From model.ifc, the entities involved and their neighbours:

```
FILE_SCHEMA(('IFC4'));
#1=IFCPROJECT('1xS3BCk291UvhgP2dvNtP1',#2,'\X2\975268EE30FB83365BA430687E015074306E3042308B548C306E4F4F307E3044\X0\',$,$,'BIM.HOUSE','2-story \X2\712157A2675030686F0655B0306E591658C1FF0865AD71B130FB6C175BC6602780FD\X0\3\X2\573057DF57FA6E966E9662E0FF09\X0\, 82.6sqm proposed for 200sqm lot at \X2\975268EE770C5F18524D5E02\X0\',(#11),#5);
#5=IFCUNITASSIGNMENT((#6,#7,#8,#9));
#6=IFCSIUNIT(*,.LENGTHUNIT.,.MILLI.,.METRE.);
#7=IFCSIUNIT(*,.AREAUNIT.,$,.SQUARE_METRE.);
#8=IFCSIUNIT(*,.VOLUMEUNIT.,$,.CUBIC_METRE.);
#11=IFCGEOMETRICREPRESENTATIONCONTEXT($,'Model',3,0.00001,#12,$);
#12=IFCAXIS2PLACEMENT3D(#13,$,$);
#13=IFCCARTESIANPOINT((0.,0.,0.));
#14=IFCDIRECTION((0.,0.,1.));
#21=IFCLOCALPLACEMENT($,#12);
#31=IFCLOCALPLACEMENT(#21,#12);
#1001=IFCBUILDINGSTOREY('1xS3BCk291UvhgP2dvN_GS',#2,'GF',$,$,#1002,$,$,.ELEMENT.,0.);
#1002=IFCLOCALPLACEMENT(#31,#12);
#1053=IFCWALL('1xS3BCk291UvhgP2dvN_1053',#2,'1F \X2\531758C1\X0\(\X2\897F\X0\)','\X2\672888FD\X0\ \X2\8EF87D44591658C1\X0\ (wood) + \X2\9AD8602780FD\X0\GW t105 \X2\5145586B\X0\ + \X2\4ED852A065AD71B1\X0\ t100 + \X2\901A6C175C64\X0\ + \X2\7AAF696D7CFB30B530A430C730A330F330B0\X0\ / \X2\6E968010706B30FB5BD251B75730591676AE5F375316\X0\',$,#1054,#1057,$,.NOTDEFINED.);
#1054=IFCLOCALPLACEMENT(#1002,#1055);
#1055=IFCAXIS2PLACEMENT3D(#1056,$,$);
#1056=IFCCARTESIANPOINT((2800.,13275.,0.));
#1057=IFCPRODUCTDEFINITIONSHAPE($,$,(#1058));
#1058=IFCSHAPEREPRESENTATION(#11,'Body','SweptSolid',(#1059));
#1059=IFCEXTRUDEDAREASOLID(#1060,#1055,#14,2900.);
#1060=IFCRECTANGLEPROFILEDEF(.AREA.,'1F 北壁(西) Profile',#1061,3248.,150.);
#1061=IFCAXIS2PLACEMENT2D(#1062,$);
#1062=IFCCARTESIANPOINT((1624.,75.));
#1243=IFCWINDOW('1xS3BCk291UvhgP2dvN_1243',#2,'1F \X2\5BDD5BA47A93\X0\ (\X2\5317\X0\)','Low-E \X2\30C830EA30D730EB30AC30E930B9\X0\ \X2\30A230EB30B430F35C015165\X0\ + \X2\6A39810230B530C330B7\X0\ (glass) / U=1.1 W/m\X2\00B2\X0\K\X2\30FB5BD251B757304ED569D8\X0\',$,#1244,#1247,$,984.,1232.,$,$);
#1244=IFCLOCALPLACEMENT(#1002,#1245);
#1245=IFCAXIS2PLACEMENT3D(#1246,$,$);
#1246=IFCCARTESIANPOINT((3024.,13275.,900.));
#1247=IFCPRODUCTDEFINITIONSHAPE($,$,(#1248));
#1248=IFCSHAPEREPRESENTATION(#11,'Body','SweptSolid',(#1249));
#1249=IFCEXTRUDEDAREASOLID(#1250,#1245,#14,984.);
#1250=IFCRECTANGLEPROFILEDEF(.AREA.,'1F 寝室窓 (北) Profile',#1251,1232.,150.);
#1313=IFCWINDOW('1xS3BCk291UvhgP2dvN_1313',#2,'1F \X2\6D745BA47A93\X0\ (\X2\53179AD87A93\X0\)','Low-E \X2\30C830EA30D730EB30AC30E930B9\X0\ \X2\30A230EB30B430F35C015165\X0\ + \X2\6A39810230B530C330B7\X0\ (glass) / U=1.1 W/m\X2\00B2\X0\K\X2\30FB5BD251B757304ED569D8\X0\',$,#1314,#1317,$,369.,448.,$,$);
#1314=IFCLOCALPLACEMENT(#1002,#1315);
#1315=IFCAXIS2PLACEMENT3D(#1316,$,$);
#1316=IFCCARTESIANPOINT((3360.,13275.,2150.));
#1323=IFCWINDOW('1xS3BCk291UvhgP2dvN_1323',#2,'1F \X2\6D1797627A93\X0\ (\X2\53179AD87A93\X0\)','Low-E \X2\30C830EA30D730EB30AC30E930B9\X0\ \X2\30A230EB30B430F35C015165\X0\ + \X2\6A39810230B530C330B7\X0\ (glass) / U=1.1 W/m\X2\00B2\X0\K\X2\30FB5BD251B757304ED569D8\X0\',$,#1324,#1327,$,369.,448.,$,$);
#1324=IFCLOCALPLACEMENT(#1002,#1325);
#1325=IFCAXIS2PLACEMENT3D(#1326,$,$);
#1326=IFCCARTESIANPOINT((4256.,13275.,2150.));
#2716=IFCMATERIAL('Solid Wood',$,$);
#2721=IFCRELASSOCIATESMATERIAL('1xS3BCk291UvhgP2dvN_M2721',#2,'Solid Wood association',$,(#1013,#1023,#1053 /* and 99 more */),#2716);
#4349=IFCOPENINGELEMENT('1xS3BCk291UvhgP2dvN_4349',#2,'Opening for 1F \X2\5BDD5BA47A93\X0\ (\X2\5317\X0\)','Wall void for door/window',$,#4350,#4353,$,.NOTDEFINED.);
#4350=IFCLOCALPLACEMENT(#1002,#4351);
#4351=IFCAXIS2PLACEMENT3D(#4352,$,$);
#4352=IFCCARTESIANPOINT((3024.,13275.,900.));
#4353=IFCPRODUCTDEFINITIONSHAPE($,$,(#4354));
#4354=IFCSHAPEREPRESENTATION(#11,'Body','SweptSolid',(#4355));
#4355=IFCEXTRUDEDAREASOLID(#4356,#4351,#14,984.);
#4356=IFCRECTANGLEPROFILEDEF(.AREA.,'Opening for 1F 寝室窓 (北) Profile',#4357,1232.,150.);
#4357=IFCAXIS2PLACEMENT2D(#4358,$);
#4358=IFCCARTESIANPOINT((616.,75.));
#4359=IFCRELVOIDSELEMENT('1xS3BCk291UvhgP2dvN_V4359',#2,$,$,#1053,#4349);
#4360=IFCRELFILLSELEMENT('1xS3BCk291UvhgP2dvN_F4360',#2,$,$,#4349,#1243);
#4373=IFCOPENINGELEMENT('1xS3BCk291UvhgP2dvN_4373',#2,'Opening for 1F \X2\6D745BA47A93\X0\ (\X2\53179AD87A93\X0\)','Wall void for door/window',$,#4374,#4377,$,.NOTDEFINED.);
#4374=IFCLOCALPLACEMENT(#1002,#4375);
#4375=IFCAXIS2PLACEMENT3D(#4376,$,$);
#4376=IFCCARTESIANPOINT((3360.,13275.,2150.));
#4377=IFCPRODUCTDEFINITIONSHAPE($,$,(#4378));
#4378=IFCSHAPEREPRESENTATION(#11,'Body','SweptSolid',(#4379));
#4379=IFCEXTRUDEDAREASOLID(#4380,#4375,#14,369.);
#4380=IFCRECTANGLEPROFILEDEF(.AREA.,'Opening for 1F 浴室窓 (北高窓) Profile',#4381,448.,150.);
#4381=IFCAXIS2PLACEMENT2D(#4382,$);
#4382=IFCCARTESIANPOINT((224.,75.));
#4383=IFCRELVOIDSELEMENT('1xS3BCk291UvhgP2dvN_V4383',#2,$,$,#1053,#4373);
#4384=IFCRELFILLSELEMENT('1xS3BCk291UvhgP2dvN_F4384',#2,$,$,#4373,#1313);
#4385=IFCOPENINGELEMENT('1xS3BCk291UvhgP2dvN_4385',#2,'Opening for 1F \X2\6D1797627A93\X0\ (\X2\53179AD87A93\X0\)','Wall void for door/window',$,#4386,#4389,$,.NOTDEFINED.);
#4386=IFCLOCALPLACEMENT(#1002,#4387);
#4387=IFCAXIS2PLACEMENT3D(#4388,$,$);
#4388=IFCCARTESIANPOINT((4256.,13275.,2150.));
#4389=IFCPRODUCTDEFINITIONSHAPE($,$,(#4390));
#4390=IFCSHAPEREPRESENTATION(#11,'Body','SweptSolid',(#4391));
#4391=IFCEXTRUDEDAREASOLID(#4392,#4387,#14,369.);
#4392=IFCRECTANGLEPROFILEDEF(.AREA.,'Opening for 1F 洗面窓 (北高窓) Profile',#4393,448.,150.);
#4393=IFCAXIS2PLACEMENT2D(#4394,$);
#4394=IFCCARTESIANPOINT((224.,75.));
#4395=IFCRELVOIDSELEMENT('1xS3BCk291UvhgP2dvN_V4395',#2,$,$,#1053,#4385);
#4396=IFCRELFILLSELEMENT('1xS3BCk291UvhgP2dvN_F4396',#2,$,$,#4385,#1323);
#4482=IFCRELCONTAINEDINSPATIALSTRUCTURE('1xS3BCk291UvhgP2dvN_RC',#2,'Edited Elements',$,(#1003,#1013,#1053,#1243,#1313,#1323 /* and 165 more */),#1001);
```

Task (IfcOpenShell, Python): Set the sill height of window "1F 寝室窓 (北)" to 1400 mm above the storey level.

```python
import numpy as np
import ifcopenshell
import ifcopenshell.api.geometry
import ifcopenshell.geom
import ifcopenshell.util.element
import ifcopenshell.util.placement
import ifcopenshell.util.shape
import ifcopenshell.util.unit

model = ifcopenshell.open("model.ifc")
unit_scale = ifcopenshell.util.unit.calculate_unit_scale(model)

window = model.by_id(1243)
opening = window.FillsVoids[0].RelatingOpeningElement
storey = ifcopenshell.util.element.get_container(window, ifc_class="IfcBuildingStorey")
level = ifcopenshell.util.placement.get_local_placement(storey.ObjectPlacement)[2, 3]

# The opening's origin need not be at the sill, so measure its lowest point.
shape = ifcopenshell.geom.create_shape(ifcopenshell.geom.settings(), opening)
bottom = ifcopenshell.util.shape.get_shape_bottom_elevation(shape, shape.geometry) / unit_scale
dz = level + 1.4 / unit_scale - bottom

shift = np.array([0.0, 0.0, dz])
# The window is not placed relative to its opening, so move both.
for product in (opening, window):
    matrix = ifcopenshell.util.placement.get_local_placement(product.ObjectPlacement)
    matrix[:3, 3] += shift
    ifcopenshell.api.geometry.edit_object_placement(model, product=product, matrix=matrix, is_si=False)

print(f"moved by {dz * unit_scale:+.3f} m")

model.write("model_rev.ifc")
```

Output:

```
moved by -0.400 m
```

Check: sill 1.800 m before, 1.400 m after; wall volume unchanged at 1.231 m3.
